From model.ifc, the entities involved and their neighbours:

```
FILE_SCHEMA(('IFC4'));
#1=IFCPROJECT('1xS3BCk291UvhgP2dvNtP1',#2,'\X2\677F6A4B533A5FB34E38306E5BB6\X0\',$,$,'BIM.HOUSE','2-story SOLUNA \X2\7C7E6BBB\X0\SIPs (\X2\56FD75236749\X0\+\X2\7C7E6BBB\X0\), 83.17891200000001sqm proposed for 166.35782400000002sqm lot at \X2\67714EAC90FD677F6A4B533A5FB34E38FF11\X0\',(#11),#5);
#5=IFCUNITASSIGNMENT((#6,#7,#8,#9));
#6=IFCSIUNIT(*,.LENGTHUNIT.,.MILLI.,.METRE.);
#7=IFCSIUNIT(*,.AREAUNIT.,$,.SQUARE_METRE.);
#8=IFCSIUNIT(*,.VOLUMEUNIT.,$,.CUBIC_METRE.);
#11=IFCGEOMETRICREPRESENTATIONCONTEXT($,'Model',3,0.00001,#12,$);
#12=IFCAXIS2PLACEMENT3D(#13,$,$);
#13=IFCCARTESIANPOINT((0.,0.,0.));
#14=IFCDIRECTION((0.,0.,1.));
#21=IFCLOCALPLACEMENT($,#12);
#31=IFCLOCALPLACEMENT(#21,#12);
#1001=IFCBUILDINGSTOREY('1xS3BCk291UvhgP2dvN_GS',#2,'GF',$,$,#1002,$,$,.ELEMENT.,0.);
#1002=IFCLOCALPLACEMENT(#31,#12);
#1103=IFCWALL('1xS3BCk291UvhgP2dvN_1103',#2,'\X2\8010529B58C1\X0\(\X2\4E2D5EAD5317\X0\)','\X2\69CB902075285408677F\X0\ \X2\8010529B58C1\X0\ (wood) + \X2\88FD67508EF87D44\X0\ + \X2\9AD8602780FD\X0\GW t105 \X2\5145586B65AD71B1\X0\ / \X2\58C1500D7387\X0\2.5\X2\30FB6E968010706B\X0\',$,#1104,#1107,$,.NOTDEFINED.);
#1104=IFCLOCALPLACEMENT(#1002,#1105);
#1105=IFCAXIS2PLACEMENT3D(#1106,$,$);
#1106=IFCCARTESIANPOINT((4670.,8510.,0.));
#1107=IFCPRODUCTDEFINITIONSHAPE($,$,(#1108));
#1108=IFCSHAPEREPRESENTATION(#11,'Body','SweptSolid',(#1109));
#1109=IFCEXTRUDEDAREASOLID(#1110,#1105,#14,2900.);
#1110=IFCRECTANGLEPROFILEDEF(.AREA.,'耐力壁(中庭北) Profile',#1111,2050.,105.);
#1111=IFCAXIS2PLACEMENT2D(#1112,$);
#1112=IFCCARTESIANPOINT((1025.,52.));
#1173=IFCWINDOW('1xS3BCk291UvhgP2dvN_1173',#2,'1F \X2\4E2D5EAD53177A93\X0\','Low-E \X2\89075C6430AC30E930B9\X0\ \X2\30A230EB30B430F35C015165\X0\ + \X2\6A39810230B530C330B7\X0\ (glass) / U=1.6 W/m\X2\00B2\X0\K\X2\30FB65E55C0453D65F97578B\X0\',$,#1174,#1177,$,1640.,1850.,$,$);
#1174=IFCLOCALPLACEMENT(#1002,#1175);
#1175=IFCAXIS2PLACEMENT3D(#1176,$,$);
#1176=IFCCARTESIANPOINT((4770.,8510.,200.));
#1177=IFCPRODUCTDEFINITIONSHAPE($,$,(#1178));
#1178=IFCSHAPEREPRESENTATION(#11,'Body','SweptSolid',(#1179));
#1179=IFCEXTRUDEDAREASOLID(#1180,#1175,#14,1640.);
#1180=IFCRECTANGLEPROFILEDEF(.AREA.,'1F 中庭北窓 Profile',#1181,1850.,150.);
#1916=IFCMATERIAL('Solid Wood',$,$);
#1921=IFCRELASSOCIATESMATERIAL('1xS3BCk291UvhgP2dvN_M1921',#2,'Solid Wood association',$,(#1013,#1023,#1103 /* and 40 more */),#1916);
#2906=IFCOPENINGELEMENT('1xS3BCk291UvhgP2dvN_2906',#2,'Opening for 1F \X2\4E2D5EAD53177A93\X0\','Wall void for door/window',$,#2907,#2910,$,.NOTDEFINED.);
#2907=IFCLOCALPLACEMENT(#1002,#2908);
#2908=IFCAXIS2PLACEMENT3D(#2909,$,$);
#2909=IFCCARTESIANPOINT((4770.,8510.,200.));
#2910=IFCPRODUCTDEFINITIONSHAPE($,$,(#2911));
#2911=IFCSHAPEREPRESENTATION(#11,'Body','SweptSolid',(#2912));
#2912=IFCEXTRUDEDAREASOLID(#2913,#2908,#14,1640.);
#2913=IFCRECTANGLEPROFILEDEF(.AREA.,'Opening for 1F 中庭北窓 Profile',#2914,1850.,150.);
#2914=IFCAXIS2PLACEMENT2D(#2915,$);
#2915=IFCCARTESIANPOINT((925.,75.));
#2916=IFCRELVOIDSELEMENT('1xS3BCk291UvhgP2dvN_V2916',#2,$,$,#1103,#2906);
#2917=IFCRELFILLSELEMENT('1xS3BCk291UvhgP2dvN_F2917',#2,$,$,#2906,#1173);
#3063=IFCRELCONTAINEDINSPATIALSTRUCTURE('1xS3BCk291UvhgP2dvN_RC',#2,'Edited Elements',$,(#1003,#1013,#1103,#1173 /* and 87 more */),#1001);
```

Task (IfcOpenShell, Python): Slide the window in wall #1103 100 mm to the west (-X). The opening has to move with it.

```python
import ifcopenshell
import ifcopenshell.api.geometry
import ifcopenshell.util.placement
import ifcopenshell.util.unit

model = ifcopenshell.open("model.ifc")
unit_scale = ifcopenshell.util.unit.calculate_unit_scale(model)

window = model.by_guid("1xS3BCk291UvhgP2dvN_1173")
opening = window.FillsVoids[0].RelatingOpeningElement
wall = opening.VoidsElements[0].RelatingBuildingElement

wall_matrix = ifcopenshell.util.placement.get_local_placement(wall.ObjectPlacement)
shift = wall_matrix[:3, 0] * -0.1 / unit_scale
before = ifcopenshell.util.placement.get_local_placement(window.ObjectPlacement)[:3, 3].copy()

# The window is not placed relative to its opening, so move both.
for product in (opening, window):
    matrix = ifcopenshell.util.placement.get_local_placement(product.ObjectPlacement)
    matrix[:3, 3] += shift
    ifcopenshell.api.geometry.edit_object_placement(model, product=product, matrix=matrix, is_si=False)

after = ifcopenshell.util.placement.get_local_placement(window.ObjectPlacement)[:3, 3]
print("window moved by", (after - before).round(3) + 0.0)

model.write("model_edited.ifc")
```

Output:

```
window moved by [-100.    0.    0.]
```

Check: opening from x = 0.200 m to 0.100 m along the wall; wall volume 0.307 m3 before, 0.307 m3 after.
